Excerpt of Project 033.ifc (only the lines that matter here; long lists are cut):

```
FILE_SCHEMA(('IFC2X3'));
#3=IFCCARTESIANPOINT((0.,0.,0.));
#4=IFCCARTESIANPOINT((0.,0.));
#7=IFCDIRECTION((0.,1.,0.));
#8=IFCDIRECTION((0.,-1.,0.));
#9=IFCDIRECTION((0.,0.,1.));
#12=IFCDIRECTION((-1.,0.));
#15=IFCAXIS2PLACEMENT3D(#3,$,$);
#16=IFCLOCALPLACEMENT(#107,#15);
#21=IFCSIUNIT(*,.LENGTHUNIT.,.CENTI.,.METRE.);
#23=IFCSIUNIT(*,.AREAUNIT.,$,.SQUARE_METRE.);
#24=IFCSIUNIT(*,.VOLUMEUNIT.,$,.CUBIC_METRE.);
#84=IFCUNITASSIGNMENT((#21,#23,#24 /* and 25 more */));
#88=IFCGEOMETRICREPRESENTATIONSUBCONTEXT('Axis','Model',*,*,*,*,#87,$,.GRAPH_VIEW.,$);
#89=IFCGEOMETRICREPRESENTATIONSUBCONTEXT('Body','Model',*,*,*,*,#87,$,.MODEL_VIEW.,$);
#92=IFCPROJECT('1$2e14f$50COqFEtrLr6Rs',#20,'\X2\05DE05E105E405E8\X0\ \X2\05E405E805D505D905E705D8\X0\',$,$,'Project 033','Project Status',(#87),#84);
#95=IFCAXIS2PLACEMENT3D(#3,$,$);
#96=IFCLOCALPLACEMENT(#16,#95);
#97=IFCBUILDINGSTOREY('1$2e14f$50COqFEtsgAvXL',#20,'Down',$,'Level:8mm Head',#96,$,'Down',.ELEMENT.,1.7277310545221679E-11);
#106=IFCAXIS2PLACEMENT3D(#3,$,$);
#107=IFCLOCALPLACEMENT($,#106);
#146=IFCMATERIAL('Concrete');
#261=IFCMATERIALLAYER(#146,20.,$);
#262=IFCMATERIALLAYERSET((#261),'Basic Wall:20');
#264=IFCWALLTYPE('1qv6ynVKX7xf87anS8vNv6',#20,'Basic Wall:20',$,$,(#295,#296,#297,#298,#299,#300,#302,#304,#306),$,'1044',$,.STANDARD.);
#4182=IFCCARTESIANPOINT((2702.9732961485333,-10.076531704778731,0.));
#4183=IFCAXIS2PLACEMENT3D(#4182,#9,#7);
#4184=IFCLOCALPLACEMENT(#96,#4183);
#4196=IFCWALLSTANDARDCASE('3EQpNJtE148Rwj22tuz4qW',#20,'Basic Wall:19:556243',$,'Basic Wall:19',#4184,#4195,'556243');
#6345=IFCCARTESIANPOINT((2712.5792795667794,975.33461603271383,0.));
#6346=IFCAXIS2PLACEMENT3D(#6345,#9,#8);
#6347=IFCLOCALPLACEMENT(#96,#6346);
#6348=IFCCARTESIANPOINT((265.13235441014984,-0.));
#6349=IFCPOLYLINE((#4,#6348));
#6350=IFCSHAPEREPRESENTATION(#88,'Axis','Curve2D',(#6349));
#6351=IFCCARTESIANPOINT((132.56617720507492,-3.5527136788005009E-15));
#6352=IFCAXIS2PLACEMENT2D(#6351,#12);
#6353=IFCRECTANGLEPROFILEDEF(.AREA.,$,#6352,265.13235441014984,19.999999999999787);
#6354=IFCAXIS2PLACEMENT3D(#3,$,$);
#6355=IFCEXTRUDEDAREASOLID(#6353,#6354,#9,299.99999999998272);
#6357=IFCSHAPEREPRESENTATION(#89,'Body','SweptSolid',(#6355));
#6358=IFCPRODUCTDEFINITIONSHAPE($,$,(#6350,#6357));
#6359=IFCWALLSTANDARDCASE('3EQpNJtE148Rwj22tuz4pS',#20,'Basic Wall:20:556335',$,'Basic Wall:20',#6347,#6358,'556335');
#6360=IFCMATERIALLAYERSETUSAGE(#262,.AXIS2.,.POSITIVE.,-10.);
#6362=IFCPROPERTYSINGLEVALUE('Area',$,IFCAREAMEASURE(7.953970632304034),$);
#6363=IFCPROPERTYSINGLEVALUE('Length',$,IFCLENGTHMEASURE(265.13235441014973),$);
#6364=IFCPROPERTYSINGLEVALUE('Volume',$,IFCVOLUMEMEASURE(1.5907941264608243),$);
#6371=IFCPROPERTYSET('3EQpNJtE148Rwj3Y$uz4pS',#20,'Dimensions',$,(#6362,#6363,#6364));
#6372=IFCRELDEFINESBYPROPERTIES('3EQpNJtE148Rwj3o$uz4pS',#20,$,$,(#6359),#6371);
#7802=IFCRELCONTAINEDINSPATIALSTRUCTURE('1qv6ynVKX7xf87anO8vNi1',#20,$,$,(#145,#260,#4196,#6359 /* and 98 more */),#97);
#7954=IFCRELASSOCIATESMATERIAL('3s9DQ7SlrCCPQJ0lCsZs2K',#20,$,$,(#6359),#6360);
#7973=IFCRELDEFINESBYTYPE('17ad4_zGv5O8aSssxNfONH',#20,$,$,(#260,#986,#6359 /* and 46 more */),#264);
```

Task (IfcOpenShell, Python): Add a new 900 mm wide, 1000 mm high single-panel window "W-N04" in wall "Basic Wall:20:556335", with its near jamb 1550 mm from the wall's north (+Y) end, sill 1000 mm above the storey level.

```python
import numpy as np
import ifcopenshell
import ifcopenshell.api.feature
import ifcopenshell.api.geometry
import ifcopenshell.api.pset
import ifcopenshell.api.root
import ifcopenshell.api.spatial
import ifcopenshell.api.type
import ifcopenshell.geom
import ifcopenshell.util.element
import ifcopenshell.util.placement
import ifcopenshell.util.representation
import ifcopenshell.util.shape
import ifcopenshell.util.unit

model = ifcopenshell.open("Project 033.ifc")
unit_scale = ifcopenshell.util.unit.calculate_unit_scale(model)
area_scale = ifcopenshell.util.unit.calculate_unit_scale(model, "AREAUNIT")
volume_scale = ifcopenshell.util.unit.calculate_unit_scale(model, "VOLUMEUNIT")
settings = ifcopenshell.geom.settings()


def volume(element):
    """Net volume in cubic metres, openings subtracted."""
    shape = ifcopenshell.geom.create_shape(settings, element)
    return ifcopenshell.util.shape.get_volume(shape.geometry)


wall = model.by_guid("3EQpNJtE148Rwj22tuz4pS")
storey = ifcopenshell.util.element.get_container(wall, ifc_class="IfcBuildingStorey")
context = ifcopenshell.util.representation.get_context(model, "Model", "Body", "MODEL_VIEW")
before = volume(wall)

width, height, from_end, sill = 0.9, 1, 1.55, 1  # metres

# The wall runs along its own X axis, and the end named is its -X end.
wall_shape = ifcopenshell.geom.create_shape(settings, wall)
x, y, z = ifcopenshell.util.shape.get_vertices(wall_shape.geometry).T
start = x.min() + from_end
face, thickness = float(y.min()), float(y.max() - y.min())
wall_matrix = ifcopenshell.util.placement.get_local_placement(wall.ObjectPlacement)
level = ifcopenshell.util.placement.get_local_placement(storey.ObjectPlacement)[2, 3]


def in_wall(x, y):
    """Placement at x, y metres in the wall's axes, at sill height."""
    matrix = wall_matrix.copy()
    matrix[:, 3] = wall_matrix @ np.array([x / unit_scale, y / unit_scale, 0.0, 1.0])
    matrix[2, 3] = level + sill / unit_scale
    return matrix


# Opening: a box that overshoots both wall faces by 50 mm.
opening = ifcopenshell.api.root.create_entity(model, ifc_class="IfcOpeningElement")
box = ifcopenshell.api.geometry.add_wall_representation(
    model, context=context, length=width, height=height, thickness=thickness + 0.1
)
ifcopenshell.api.geometry.assign_representation(model, product=opening, representation=box)
ifcopenshell.api.geometry.edit_object_placement(model, product=opening, matrix=in_wall(start, face - 0.05), is_si=False)
ifcopenshell.api.feature.add_feature(model, feature=opening, element=wall)

window = ifcopenshell.api.root.create_entity(model, ifc_class="IfcWindow", name="W-N04")
window.OverallWidth, window.OverallHeight = width / unit_scale, height / unit_scale
body = ifcopenshell.api.geometry.add_window_representation(
    model,
    context=context,
    overall_width=window.OverallWidth,
    overall_height=window.OverallHeight,
    partition_type="SINGLE_PANEL",
)
ifcopenshell.api.geometry.assign_representation(model, product=window, representation=body)
ifcopenshell.api.spatial.assign_container(model, products=[window], relating_structure=storey)
fills = ifcopenshell.api.feature.add_filling(model, opening=opening, element=window)
fills.OwnerHistory = window.OwnerHistory  # required in IFC2X3

# IFC2X3 keeps the operation on the window style.
style = ifcopenshell.api.root.create_entity(model, ifc_class="IfcWindowStyle", name="W-N04")
style.OperationType, style.ConstructionType = "SINGLE_PANEL", "NOTDEFINED"
style.ParameterTakesPrecedence = style.Sizeable = False
ifcopenshell.api.type.assign_type(model, related_objects=[window], relating_type=style)

# Centre the window in the wall's thickness.
ifcopenshell.api.geometry.edit_object_placement(model, product=window, matrix=in_wall(start, face), is_si=False)
window_shape = ifcopenshell.geom.create_shape(settings, window)
depth = ifcopenshell.util.shape.get_vertices(window_shape.geometry)[:, 1]
offset = face + thickness / 2 - (depth.min() + depth.max()) / 2
ifcopenshell.api.geometry.edit_object_placement(model, product=window, matrix=in_wall(start, offset), is_si=False)

after = volume(wall)

# Update the wall's stored quantities.
pset = model.by_id(ifcopenshell.util.element.get_pset(wall, "Dimensions", should_inherit=False)["id"])
ifcopenshell.api.pset.edit_pset(model, pset=pset, properties={
    "Area": model.create_entity("IfcAreaMeasure", after / thickness / area_scale),
    "Volume": model.create_entity("IfcVolumeMeasure", after / volume_scale),
})

print(f"wall volume {before:.3f} -> {after:.3f} m3")

model.write("Project 033-out.ifc")
```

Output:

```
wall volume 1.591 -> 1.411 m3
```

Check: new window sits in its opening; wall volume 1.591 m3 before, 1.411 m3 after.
